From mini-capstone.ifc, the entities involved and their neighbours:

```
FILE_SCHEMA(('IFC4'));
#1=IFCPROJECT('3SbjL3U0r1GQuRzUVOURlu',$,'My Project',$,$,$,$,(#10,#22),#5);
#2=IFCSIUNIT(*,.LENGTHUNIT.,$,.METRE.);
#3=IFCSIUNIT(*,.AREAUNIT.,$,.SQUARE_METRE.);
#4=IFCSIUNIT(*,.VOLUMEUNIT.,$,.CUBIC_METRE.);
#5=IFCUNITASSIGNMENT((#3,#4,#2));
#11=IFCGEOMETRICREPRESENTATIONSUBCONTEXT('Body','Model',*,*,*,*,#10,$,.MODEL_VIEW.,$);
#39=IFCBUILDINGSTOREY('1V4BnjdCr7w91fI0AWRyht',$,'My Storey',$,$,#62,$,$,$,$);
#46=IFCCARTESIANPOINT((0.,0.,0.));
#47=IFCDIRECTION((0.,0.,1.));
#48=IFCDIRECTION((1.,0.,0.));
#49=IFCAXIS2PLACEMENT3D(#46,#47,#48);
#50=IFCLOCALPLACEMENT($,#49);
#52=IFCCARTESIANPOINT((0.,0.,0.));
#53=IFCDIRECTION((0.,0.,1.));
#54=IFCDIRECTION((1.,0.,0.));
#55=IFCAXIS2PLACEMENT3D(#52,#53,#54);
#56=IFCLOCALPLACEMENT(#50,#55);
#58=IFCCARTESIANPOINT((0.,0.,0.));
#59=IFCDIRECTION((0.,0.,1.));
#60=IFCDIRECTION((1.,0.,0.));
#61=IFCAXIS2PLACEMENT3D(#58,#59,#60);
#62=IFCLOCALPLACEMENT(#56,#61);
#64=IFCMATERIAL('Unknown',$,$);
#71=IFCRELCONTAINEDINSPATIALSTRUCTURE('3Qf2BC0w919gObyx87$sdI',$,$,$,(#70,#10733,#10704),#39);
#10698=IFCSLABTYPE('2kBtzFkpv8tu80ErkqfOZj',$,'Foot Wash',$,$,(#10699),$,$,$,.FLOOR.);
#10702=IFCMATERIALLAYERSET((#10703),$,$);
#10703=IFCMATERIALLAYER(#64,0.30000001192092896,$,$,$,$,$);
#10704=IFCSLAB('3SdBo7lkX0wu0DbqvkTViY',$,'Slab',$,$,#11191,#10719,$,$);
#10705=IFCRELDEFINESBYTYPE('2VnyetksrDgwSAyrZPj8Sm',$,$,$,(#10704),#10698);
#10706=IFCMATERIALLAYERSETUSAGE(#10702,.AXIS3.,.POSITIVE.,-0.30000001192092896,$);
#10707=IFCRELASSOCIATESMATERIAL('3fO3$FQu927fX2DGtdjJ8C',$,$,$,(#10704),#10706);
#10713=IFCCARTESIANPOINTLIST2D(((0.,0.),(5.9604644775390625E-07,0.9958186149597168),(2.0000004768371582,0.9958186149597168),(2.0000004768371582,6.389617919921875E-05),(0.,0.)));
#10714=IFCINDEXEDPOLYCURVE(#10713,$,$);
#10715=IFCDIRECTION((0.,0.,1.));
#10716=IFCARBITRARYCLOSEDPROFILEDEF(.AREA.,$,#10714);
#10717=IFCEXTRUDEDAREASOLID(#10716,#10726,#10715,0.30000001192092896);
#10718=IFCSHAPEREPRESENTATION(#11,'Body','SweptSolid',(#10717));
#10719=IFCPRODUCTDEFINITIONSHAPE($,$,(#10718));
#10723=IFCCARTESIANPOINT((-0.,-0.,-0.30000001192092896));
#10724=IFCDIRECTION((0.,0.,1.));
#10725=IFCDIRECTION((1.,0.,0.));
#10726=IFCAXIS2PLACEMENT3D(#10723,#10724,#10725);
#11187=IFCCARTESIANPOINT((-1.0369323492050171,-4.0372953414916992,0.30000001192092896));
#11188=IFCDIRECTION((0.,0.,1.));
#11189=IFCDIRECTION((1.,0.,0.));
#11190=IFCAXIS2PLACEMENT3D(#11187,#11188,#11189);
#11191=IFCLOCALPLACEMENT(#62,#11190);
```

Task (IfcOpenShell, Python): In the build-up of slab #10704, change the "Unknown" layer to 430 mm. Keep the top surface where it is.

```python
import ifcopenshell
import ifcopenshell.util.element
import ifcopenshell.util.representation
import ifcopenshell.util.unit

model = ifcopenshell.open("mini-capstone.ifc")
unit_scale = ifcopenshell.util.unit.calculate_unit_scale(model)

layer_set = model.by_id(10702)
layer = next(l for l in layer_set.MaterialLayers if l.Material and l.Material.Name == "Unknown")
change = 0.43 / unit_scale - layer.LayerThickness
layer.LayerThickness += change

# Geometry does not follow the layer set by itself.
slabs = [e for e in ifcopenshell.util.element.get_elements_by_material(model, layer_set) if e.is_a("IfcSlab")]
for slab in sorted(slabs, key=lambda e: e.id()):
    body = ifcopenshell.util.representation.get_representation(slab, "Model", "Body")
    solid = body.Items[0]
    old_depth = solid.Depth
    solid.Depth += change
    # Extruded upwards: lower the start of the extrusion so the top stays.
    x, y, z = solid.Position.Location.Coordinates
    solid.Position.Location = model.createIfcCartesianPoint((x, y, z - change))
    print(slab.id(), f"{old_depth:g} -> {solid.Depth:g}")

# The layers are counted up from the underside, which has moved.
for usage in {ifcopenshell.util.element.get_material(slab) for slab in slabs}:
    usage.OffsetFromReferenceLine -= change

model.write("mini-capstone_v2.ifc")
```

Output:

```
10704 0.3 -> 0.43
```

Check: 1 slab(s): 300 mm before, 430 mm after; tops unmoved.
